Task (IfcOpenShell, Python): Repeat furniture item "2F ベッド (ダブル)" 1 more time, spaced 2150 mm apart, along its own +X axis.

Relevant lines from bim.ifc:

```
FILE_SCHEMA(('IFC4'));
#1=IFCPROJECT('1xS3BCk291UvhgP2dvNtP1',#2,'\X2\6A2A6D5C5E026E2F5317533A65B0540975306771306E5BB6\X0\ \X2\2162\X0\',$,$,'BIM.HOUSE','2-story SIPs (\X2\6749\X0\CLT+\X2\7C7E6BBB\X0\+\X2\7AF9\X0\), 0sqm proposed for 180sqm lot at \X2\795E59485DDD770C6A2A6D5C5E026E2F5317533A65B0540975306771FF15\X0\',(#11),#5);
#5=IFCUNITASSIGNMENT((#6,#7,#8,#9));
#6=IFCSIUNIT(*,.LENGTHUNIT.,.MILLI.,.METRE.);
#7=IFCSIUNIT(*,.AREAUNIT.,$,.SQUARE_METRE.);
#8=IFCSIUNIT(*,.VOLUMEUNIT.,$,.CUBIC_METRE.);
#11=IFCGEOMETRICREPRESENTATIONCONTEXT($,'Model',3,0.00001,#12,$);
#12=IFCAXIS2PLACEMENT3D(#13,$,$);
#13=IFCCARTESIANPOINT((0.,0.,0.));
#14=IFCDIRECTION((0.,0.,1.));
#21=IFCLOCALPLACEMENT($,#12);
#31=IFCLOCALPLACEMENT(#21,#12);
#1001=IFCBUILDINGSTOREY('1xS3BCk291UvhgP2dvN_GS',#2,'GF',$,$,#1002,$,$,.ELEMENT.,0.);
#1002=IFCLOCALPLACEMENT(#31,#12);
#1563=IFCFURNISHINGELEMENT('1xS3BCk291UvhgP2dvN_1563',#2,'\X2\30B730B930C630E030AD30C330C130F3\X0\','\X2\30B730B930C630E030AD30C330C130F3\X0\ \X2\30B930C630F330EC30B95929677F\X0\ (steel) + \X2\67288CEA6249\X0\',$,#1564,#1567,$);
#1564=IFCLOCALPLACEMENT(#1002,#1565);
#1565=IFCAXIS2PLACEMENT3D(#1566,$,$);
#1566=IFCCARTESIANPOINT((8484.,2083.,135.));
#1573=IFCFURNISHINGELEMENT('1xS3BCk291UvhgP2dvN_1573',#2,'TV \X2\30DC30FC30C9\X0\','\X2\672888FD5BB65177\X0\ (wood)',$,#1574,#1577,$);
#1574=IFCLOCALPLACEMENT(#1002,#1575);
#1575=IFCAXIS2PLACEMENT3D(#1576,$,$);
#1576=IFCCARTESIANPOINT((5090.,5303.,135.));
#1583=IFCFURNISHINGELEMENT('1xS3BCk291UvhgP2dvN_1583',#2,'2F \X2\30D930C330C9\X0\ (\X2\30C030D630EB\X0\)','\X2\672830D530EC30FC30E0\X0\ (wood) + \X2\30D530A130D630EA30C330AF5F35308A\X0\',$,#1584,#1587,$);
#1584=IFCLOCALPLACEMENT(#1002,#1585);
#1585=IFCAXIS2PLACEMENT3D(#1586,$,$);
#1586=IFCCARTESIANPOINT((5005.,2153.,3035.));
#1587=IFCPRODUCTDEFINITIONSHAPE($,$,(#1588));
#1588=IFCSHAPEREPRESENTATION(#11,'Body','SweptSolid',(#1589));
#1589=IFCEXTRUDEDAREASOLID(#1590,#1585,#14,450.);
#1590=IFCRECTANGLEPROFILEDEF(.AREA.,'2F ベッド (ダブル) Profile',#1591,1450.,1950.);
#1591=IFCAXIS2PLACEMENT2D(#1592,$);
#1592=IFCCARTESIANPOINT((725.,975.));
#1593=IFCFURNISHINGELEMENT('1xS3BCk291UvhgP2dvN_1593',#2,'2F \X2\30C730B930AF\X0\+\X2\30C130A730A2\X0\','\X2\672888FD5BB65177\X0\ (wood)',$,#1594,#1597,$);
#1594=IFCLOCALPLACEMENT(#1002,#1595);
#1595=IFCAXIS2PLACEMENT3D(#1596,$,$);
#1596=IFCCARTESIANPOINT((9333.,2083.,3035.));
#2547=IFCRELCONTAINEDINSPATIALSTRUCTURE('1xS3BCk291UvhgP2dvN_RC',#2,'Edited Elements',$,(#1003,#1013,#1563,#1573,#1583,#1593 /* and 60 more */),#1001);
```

```python
import ifcopenshell
import ifcopenshell.api.geometry
import ifcopenshell.api.root
import ifcopenshell.util.element
import ifcopenshell.util.placement
import ifcopenshell.util.unit

model = ifcopenshell.open("bim.ifc")
unit_scale = ifcopenshell.util.unit.calculate_unit_scale(model)


def reuse_history(source, copy):
    """copy_class also copies each property set's owner history, people and application; keep the originals."""
    for rel in copy.IsDefinedBy:
        if rel.is_a("IfcRelDefinesByProperties") and (history := rel.RelatingPropertyDefinition.OwnerHistory):
            rel.RelatingPropertyDefinition.OwnerHistory = source.OwnerHistory
            ifcopenshell.util.element.remove_deep2(model, history)


source = model.by_guid("1xS3BCk291UvhgP2dvN_1583")
base = ifcopenshell.util.placement.get_local_placement(source.ObjectPlacement)
step = base[:3, 0] * 2.15 / unit_scale

for i in range(1, 2):
    copy = ifcopenshell.api.root.copy_class(model, product=source)
    copy.Representation = ifcopenshell.util.element.copy_deep(
        model, source.Representation, exclude=["IfcGeometricRepresentationContext", "IfcRepresentationMap"]
    )
    reuse_history(source, copy)
    matrix = base.copy()
    matrix[:3, 3] += i * step
    print("added at", matrix[:3, 3].round(3) + 0.0)
    ifcopenshell.api.geometry.edit_object_placement(model, product=copy, matrix=matrix, is_si=False)

model.write("bim_edited.ifc")
```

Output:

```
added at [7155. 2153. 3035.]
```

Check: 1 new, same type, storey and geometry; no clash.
